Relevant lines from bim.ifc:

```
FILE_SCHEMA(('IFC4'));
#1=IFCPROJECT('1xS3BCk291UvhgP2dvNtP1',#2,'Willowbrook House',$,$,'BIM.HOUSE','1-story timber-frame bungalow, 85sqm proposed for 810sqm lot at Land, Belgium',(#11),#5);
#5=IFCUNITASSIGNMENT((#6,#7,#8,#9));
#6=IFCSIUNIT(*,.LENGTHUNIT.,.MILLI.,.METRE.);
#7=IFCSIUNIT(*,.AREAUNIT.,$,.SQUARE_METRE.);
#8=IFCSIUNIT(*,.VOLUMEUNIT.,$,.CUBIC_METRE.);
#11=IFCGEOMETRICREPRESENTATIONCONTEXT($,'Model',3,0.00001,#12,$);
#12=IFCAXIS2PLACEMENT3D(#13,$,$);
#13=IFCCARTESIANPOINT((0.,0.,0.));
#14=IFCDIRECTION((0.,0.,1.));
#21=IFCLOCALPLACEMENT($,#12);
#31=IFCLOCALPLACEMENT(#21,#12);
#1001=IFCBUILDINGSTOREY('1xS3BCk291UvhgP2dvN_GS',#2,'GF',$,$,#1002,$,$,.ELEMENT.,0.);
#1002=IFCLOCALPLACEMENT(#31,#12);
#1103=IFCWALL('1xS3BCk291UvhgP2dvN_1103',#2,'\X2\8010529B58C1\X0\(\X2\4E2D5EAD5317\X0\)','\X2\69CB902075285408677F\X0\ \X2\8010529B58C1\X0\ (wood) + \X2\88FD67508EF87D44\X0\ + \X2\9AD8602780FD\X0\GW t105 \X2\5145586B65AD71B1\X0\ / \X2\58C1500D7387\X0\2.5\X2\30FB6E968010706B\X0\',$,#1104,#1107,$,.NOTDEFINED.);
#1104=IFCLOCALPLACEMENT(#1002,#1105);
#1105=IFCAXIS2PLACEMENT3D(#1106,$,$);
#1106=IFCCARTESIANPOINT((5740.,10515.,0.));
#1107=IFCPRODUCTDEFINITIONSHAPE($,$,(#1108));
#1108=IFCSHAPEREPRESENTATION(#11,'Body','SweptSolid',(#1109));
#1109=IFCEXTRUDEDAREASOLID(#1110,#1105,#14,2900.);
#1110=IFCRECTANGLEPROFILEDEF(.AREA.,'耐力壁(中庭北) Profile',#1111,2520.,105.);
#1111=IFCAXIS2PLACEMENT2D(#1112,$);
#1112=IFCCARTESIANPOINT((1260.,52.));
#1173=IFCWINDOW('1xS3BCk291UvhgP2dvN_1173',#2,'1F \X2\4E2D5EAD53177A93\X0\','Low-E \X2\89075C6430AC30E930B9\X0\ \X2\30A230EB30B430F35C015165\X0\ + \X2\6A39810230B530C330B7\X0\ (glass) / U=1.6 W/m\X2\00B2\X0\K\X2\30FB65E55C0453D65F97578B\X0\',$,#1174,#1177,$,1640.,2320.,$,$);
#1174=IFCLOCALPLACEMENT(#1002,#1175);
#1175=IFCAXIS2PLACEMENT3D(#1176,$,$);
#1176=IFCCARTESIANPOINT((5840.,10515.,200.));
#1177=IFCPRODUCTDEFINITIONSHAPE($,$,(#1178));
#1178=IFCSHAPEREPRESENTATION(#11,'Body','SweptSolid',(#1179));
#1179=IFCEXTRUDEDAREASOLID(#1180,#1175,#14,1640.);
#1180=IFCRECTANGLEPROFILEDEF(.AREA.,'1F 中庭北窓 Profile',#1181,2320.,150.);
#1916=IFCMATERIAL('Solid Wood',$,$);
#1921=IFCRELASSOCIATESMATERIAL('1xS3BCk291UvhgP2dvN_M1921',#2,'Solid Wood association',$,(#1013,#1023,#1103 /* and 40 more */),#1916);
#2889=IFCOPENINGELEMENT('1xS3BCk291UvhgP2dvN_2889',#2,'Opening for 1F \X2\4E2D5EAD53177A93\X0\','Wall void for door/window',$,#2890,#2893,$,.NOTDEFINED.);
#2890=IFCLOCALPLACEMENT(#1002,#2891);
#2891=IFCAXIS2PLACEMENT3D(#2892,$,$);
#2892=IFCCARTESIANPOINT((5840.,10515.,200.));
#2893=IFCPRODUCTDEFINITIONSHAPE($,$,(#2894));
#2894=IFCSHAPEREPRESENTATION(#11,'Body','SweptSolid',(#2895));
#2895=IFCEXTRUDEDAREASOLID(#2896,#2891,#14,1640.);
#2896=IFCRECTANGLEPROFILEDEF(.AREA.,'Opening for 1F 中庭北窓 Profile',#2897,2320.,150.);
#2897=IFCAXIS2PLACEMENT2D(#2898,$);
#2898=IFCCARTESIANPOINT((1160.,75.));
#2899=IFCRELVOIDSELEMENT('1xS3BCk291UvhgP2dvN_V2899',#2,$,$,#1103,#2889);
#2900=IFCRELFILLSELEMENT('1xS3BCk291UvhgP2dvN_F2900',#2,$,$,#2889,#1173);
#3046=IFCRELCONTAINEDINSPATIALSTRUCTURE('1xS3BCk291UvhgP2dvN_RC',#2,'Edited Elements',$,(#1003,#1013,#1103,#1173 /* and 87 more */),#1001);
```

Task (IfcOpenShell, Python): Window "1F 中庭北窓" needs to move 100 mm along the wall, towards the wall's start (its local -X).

```python
import ifcopenshell
import ifcopenshell.api.geometry
import ifcopenshell.util.placement
import ifcopenshell.util.unit

model = ifcopenshell.open("bim.ifc")
unit_scale = ifcopenshell.util.unit.calculate_unit_scale(model)

window = model.by_guid("1xS3BCk291UvhgP2dvN_1173")
opening = window.FillsVoids[0].RelatingOpeningElement
wall = opening.VoidsElements[0].RelatingBuildingElement

wall_matrix = ifcopenshell.util.placement.get_local_placement(wall.ObjectPlacement)
shift = wall_matrix[:3, 0] * -0.1 / unit_scale
before = ifcopenshell.util.placement.get_local_placement(window.ObjectPlacement)[:3, 3].copy()

# The window is not placed relative to its opening, so move both.
for product in (opening, window):
    matrix = ifcopenshell.util.placement.get_local_placement(product.ObjectPlacement)
    matrix[:3, 3] += shift
    ifcopenshell.api.geometry.edit_object_placement(model, product=product, matrix=matrix, is_si=False)

after = ifcopenshell.util.placement.get_local_placement(window.ObjectPlacement)[:3, 3]
print("window moved by", (after - before).round(3) + 0.0)

model.write("bim_edited.ifc")
```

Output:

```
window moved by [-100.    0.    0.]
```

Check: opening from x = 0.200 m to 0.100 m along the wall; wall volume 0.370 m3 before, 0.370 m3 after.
